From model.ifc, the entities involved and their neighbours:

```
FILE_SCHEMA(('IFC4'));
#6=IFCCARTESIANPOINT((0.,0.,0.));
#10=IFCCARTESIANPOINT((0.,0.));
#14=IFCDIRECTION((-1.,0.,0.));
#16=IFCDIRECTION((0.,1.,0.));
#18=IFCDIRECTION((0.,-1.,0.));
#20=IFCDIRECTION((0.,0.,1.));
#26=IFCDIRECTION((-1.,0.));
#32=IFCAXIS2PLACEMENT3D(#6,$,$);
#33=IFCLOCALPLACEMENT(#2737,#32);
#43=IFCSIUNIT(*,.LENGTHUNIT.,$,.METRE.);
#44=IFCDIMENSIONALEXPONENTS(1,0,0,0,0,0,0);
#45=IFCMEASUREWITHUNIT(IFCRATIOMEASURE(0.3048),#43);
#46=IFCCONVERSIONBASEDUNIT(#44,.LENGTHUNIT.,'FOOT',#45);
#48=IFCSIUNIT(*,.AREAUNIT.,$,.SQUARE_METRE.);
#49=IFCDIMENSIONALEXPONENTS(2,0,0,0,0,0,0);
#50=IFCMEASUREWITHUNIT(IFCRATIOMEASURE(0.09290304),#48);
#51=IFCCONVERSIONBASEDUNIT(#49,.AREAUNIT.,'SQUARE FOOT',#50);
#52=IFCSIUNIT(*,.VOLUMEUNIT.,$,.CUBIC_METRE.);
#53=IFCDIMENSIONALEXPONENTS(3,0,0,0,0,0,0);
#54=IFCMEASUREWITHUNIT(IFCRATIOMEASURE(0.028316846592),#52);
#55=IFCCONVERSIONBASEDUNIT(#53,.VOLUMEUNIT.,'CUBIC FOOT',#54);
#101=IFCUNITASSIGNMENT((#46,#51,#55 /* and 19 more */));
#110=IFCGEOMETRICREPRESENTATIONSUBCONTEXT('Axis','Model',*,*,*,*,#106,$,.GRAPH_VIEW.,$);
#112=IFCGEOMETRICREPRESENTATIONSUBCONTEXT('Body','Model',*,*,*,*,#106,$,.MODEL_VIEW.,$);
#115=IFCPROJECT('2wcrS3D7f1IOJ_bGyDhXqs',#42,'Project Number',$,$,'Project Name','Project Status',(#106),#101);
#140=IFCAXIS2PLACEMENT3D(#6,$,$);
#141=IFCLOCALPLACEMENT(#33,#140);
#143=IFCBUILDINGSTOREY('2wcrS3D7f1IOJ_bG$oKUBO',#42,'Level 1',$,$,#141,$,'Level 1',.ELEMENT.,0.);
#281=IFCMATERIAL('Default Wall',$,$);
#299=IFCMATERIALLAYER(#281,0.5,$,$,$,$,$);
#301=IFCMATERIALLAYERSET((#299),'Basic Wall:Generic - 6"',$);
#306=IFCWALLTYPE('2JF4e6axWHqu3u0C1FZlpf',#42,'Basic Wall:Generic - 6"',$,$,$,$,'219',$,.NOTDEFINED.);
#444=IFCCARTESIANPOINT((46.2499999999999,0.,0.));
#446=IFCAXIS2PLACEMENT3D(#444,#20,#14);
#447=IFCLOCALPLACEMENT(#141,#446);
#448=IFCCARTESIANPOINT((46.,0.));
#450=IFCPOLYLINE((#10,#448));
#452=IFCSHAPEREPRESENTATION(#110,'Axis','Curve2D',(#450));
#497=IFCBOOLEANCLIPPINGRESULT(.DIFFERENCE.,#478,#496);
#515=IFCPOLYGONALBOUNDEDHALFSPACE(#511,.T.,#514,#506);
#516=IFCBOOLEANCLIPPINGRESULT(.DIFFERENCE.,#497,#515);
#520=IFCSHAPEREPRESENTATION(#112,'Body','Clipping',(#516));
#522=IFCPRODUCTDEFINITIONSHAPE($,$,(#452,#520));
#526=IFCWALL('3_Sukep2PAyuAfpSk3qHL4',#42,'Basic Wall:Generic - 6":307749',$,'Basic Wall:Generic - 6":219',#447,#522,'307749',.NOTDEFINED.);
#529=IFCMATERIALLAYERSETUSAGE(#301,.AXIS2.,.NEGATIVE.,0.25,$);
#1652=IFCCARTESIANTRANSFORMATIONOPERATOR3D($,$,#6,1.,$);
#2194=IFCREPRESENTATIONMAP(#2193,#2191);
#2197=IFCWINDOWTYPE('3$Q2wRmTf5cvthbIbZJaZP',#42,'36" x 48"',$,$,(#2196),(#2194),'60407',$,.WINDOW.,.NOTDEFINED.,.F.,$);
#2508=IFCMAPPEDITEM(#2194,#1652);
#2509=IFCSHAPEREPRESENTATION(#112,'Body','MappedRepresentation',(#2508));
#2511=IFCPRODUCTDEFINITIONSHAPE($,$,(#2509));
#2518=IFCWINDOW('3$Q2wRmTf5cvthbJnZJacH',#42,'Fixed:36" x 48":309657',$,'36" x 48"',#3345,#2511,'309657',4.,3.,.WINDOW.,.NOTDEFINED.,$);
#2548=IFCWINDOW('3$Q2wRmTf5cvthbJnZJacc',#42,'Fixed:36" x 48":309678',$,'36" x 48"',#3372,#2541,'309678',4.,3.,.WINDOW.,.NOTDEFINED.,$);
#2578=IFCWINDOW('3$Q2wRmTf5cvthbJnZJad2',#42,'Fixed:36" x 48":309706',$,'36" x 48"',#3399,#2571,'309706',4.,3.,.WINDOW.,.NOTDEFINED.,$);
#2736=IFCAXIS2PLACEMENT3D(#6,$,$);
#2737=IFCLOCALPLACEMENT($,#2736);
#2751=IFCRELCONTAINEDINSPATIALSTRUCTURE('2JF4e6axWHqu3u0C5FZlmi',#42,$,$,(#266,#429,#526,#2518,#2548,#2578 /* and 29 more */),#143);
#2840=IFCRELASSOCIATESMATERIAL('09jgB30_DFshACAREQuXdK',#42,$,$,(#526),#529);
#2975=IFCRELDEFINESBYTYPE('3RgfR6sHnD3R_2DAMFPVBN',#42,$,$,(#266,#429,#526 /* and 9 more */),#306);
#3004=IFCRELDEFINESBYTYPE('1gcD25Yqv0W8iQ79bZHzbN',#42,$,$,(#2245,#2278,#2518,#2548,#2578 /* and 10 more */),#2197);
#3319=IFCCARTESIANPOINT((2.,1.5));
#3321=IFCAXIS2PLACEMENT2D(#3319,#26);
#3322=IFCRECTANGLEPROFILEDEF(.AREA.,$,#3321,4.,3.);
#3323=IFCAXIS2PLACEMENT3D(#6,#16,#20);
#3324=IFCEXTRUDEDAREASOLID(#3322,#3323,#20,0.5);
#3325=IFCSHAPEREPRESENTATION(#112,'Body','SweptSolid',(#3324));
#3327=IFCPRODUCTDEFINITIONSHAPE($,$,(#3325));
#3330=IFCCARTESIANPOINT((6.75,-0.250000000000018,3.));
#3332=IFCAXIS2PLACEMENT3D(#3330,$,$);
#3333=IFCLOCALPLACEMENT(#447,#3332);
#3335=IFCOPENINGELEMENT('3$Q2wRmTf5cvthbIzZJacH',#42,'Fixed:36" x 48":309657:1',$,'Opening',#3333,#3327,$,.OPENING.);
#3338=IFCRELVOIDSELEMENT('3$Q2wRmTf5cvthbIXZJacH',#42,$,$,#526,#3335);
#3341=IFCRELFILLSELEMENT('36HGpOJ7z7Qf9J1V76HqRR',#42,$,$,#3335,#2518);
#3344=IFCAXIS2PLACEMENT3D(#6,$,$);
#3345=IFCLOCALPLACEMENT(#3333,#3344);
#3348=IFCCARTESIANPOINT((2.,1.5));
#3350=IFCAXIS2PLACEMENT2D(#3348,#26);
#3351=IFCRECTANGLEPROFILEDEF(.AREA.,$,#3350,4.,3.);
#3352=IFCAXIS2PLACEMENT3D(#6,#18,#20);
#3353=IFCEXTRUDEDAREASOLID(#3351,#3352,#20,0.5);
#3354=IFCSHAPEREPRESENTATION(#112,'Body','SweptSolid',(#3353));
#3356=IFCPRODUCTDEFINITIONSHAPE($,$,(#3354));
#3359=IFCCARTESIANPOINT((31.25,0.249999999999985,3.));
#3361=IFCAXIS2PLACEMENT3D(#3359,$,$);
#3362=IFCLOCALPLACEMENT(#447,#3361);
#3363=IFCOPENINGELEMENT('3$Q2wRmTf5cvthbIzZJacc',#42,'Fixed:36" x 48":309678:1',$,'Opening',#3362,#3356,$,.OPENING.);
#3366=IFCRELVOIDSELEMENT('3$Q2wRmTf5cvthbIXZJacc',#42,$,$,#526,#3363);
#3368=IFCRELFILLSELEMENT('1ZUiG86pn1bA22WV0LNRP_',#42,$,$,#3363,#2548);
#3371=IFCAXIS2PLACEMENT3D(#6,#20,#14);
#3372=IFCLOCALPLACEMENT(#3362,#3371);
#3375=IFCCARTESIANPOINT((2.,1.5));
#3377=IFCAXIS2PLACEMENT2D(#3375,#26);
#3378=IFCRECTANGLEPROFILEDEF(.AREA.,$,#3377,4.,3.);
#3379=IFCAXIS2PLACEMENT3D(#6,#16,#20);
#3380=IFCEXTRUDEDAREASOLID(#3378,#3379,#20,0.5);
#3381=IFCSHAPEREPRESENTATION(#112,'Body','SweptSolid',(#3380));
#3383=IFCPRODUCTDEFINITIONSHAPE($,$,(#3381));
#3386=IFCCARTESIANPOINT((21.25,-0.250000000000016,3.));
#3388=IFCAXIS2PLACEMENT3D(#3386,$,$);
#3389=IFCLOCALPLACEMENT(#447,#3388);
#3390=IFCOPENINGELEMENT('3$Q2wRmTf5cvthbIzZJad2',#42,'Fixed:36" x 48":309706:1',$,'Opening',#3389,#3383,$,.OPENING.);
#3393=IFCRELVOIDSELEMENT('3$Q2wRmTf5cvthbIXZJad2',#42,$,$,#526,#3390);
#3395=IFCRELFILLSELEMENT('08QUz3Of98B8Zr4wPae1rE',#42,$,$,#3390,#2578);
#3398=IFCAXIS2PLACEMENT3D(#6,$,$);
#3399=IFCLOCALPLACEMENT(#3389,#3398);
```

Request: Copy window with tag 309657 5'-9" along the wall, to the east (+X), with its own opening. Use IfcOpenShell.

```python
import ifcopenshell
import ifcopenshell.api.feature
import ifcopenshell.api.geometry
import ifcopenshell.api.root
import ifcopenshell.geom
import ifcopenshell.util.element
import ifcopenshell.util.placement
import ifcopenshell.util.shape
import ifcopenshell.util.unit

model = ifcopenshell.open("model.ifc")
unit_scale = ifcopenshell.util.unit.calculate_unit_scale(model)
settings = ifcopenshell.geom.settings()


def volume(element):
    """Net volume in cubic metres, openings subtracted."""
    shape = ifcopenshell.geom.create_shape(settings, element)
    return ifcopenshell.util.shape.get_volume(shape.geometry)


def reuse_history(source, copy):
    """copy_class also copies each property set's owner history, people and application; keep the originals."""
    for rel in copy.IsDefinedBy:
        if rel.is_a("IfcRelDefinesByProperties") and (history := rel.RelatingPropertyDefinition.OwnerHistory):
            rel.RelatingPropertyDefinition.OwnerHistory = source.OwnerHistory
            ifcopenshell.util.element.remove_deep2(model, history)


window = model.by_guid("3$Q2wRmTf5cvthbJnZJacH")
opening = window.FillsVoids[0].RelatingOpeningElement
wall = opening.VoidsElements[0].RelatingBuildingElement
before = volume(wall)
shift = ifcopenshell.util.placement.get_local_placement(wall.ObjectPlacement)[:3, 0] * -69 * 0.0254 / unit_scale

# copy_class copies the void relationship, type, container and properties, but no geometry.
new_opening = ifcopenshell.api.root.copy_class(model, product=opening)
new_opening.Representation = ifcopenshell.util.element.copy_deep(
    model, opening.Representation, exclude=["IfcGeometricRepresentationContext", "IfcRepresentationMap"]
)
new_opening.Name = 'Fixed:36" x 48"'
new_window = ifcopenshell.api.root.copy_class(model, product=window)
new_window.Representation = ifcopenshell.util.element.copy_deep(
    model, window.Representation, exclude=["IfcGeometricRepresentationContext", "IfcRepresentationMap"]
)
new_window.Name = 'Fixed:36" x 48"'
new_window.Tag = None
reuse_history(window, new_window)
ifcopenshell.api.feature.add_filling(model, opening=new_opening, element=new_window)

for old, new in ((opening, new_opening), (window, new_window)):
    matrix = ifcopenshell.util.placement.get_local_placement(old.ObjectPlacement)
    matrix[:3, 3] += shift
    ifcopenshell.api.geometry.edit_object_placement(model, product=new, matrix=matrix, is_si=False)

after = volume(wall)

print(f"wall volume {before:.3f} -> {after:.3f} m3")

model.write("model_edited.ifc")
```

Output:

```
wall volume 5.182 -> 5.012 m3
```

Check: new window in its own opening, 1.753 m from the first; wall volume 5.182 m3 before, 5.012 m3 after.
